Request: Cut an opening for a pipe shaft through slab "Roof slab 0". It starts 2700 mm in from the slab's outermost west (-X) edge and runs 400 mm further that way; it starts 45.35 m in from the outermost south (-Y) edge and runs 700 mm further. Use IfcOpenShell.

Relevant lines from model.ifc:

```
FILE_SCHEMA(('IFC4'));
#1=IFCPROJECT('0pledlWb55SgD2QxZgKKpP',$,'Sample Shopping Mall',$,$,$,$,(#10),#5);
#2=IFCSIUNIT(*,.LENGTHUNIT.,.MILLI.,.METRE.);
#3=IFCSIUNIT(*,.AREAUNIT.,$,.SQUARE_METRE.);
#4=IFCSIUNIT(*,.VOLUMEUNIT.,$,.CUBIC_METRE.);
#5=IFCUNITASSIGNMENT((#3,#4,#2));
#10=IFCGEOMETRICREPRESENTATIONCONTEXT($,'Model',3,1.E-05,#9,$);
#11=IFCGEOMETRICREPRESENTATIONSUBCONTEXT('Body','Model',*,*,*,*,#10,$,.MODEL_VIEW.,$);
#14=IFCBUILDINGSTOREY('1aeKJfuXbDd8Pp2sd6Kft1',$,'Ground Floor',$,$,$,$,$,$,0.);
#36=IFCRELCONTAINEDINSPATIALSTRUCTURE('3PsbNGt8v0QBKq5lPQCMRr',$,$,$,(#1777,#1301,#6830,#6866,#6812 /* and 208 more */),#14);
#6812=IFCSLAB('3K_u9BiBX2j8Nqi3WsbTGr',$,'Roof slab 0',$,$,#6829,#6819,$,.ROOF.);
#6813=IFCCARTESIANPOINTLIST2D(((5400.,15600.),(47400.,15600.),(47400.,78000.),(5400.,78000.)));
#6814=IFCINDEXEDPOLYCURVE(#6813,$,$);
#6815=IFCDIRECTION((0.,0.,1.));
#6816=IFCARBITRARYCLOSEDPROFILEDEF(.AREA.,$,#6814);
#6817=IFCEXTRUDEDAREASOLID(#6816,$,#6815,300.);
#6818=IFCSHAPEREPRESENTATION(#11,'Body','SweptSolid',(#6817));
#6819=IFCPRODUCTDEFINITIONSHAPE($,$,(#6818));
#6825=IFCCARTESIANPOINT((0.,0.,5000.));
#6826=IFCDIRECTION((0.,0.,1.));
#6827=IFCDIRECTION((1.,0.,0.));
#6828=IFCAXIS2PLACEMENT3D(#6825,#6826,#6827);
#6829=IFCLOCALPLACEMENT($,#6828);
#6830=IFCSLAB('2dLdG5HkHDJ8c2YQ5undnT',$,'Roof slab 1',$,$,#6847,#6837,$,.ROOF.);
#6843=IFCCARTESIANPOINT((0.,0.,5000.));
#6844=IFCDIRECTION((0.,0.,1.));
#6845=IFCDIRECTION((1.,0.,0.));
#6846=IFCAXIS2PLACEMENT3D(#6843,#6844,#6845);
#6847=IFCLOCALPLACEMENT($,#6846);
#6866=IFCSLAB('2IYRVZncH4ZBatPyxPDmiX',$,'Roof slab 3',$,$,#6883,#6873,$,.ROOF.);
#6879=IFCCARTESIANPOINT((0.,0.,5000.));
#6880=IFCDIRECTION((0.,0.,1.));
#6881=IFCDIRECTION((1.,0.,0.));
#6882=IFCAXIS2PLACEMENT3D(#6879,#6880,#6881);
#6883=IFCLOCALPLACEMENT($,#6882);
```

```python
import numpy as np
import ifcopenshell
import ifcopenshell.api.feature
import ifcopenshell.api.geometry
import ifcopenshell.api.root
import ifcopenshell.geom
import ifcopenshell.util.placement
import ifcopenshell.util.representation
import ifcopenshell.util.shape
import ifcopenshell.util.unit

model = ifcopenshell.open("model.ifc")
unit_scale = ifcopenshell.util.unit.calculate_unit_scale(model)
settings = ifcopenshell.geom.settings()


def volume(element):
    """Net volume in cubic metres, openings subtracted."""
    shape = ifcopenshell.geom.create_shape(settings, element)
    return ifcopenshell.util.shape.get_volume(shape.geometry)


slab = model.by_guid("3K_u9BiBX2j8Nqi3WsbTGr")
before = volume(slab)

# Extent in the slab's own axes, in metres. The edges named are its -X and -Y sides.
slab_shape = ifcopenshell.geom.create_shape(settings, slab)
vertices = ifcopenshell.util.shape.get_vertices(slab_shape.geometry)
x_min, y_min, bottom = vertices.min(axis=0)
top = vertices[:, 2].max()

opening = ifcopenshell.api.root.create_entity(model, ifc_class="IfcOpeningElement", name="Pipe shaft opening", predefined_type="OPENING")
context = ifcopenshell.util.representation.get_context(model, "Model", "Body", "MODEL_VIEW")
width, depth = 0.4, 0.7
outline = [(0.0, 0.0), (width, 0.0), (width, depth), (0.0, depth), (0.0, 0.0)]
# Overshoot both faces by 50 mm so the cut is clean.
shape = ifcopenshell.api.geometry.add_slab_representation(
    model, context=context, depth=top - bottom + 0.1, polyline=outline
)
ifcopenshell.api.geometry.assign_representation(model, product=opening, representation=shape)

matrix = ifcopenshell.util.placement.get_local_placement(slab.ObjectPlacement)
matrix[:, 3] = matrix @ np.append(np.array([x_min + 2.7, y_min + 45.35, bottom - 0.05]) / unit_scale, 1.0)
ifcopenshell.api.geometry.edit_object_placement(model, product=opening, matrix=matrix, is_si=False)
ifcopenshell.api.feature.add_feature(model, feature=opening, element=slab)

after = volume(slab)

print(f"slab volume {before:.3f} -> {after:.3f} m3")

model.write("model_rev.ifc")
```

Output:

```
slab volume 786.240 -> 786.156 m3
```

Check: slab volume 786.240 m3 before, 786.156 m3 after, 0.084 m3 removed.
